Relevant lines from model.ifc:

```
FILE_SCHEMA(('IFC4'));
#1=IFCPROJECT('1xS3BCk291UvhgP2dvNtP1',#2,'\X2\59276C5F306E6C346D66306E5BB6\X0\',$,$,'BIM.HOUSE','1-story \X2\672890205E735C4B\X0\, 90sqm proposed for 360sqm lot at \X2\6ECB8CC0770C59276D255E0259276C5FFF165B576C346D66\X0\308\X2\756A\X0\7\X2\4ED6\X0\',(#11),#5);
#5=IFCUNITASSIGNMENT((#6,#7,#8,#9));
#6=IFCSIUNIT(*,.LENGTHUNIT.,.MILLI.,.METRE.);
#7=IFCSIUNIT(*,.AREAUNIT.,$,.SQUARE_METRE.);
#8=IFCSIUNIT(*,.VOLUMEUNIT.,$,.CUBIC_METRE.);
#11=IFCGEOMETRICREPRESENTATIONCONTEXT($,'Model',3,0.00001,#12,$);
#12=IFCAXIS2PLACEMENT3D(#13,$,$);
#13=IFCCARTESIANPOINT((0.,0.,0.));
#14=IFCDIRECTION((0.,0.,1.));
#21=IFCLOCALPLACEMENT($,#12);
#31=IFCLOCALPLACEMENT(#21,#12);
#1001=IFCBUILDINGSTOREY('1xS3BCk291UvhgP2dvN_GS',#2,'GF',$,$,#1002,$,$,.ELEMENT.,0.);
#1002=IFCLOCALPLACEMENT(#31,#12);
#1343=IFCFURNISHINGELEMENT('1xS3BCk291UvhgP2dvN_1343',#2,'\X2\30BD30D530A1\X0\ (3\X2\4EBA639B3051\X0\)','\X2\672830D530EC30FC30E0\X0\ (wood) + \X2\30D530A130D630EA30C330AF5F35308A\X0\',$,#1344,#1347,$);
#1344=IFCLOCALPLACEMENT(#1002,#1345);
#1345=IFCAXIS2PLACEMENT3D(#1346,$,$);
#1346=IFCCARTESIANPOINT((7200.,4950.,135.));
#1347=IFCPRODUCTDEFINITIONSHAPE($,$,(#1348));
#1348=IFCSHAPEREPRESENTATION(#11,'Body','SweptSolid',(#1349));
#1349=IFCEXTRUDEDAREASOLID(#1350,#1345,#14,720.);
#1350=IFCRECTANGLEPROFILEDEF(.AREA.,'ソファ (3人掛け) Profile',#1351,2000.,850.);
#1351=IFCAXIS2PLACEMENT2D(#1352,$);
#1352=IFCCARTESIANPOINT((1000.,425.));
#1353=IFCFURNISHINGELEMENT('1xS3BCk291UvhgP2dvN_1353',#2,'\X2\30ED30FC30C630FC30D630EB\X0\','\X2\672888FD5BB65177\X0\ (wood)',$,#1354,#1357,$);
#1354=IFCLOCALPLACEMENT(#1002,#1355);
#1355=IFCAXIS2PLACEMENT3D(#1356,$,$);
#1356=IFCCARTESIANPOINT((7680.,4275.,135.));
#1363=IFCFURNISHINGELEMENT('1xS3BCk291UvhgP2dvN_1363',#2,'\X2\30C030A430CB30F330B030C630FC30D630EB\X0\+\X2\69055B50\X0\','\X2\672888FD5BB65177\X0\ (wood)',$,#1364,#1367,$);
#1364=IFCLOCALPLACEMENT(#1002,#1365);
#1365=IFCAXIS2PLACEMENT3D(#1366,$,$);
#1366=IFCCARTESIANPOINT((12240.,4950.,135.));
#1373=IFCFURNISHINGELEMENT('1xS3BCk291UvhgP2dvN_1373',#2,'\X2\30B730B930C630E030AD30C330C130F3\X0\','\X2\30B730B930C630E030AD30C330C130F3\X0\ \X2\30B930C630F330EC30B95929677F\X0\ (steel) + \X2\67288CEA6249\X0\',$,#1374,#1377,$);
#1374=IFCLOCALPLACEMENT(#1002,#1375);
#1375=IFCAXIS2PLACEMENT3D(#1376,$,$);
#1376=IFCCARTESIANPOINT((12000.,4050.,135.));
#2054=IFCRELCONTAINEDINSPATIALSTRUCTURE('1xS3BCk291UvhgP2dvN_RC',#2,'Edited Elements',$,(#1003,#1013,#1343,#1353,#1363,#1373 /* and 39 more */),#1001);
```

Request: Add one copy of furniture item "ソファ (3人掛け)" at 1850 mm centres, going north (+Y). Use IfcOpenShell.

```python
import numpy as np
import ifcopenshell
import ifcopenshell.api.geometry
import ifcopenshell.api.root
import ifcopenshell.util.element
import ifcopenshell.util.placement

model = ifcopenshell.open("model.ifc")


def reuse_history(source, copy):
    """copy_class also copies each property set's owner history, people and application; keep the originals."""
    for rel in copy.IsDefinedBy:
        if rel.is_a("IfcRelDefinesByProperties") and (history := rel.RelatingPropertyDefinition.OwnerHistory):
            rel.RelatingPropertyDefinition.OwnerHistory = source.OwnerHistory
            ifcopenshell.util.element.remove_deep2(model, history)


source = model.by_id(1343)
base = ifcopenshell.util.placement.get_local_placement(source.ObjectPlacement)
step = np.array([0.0, 1.0, 0.0]) * 1850.0

for i in range(1, 2):
    copy = ifcopenshell.api.root.copy_class(model, product=source)
    copy.Representation = ifcopenshell.util.element.copy_deep(
        model, source.Representation, exclude=["IfcGeometricRepresentationContext", "IfcRepresentationMap"]
    )
    reuse_history(source, copy)
    matrix = base.copy()
    matrix[:3, 3] += i * step
    print("added at", matrix[:3, 3].round(3) + 0.0)
    ifcopenshell.api.geometry.edit_object_placement(model, product=copy, matrix=matrix, is_si=False)

model.write("model_v2.ifc")
```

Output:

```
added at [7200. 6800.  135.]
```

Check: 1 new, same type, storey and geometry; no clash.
